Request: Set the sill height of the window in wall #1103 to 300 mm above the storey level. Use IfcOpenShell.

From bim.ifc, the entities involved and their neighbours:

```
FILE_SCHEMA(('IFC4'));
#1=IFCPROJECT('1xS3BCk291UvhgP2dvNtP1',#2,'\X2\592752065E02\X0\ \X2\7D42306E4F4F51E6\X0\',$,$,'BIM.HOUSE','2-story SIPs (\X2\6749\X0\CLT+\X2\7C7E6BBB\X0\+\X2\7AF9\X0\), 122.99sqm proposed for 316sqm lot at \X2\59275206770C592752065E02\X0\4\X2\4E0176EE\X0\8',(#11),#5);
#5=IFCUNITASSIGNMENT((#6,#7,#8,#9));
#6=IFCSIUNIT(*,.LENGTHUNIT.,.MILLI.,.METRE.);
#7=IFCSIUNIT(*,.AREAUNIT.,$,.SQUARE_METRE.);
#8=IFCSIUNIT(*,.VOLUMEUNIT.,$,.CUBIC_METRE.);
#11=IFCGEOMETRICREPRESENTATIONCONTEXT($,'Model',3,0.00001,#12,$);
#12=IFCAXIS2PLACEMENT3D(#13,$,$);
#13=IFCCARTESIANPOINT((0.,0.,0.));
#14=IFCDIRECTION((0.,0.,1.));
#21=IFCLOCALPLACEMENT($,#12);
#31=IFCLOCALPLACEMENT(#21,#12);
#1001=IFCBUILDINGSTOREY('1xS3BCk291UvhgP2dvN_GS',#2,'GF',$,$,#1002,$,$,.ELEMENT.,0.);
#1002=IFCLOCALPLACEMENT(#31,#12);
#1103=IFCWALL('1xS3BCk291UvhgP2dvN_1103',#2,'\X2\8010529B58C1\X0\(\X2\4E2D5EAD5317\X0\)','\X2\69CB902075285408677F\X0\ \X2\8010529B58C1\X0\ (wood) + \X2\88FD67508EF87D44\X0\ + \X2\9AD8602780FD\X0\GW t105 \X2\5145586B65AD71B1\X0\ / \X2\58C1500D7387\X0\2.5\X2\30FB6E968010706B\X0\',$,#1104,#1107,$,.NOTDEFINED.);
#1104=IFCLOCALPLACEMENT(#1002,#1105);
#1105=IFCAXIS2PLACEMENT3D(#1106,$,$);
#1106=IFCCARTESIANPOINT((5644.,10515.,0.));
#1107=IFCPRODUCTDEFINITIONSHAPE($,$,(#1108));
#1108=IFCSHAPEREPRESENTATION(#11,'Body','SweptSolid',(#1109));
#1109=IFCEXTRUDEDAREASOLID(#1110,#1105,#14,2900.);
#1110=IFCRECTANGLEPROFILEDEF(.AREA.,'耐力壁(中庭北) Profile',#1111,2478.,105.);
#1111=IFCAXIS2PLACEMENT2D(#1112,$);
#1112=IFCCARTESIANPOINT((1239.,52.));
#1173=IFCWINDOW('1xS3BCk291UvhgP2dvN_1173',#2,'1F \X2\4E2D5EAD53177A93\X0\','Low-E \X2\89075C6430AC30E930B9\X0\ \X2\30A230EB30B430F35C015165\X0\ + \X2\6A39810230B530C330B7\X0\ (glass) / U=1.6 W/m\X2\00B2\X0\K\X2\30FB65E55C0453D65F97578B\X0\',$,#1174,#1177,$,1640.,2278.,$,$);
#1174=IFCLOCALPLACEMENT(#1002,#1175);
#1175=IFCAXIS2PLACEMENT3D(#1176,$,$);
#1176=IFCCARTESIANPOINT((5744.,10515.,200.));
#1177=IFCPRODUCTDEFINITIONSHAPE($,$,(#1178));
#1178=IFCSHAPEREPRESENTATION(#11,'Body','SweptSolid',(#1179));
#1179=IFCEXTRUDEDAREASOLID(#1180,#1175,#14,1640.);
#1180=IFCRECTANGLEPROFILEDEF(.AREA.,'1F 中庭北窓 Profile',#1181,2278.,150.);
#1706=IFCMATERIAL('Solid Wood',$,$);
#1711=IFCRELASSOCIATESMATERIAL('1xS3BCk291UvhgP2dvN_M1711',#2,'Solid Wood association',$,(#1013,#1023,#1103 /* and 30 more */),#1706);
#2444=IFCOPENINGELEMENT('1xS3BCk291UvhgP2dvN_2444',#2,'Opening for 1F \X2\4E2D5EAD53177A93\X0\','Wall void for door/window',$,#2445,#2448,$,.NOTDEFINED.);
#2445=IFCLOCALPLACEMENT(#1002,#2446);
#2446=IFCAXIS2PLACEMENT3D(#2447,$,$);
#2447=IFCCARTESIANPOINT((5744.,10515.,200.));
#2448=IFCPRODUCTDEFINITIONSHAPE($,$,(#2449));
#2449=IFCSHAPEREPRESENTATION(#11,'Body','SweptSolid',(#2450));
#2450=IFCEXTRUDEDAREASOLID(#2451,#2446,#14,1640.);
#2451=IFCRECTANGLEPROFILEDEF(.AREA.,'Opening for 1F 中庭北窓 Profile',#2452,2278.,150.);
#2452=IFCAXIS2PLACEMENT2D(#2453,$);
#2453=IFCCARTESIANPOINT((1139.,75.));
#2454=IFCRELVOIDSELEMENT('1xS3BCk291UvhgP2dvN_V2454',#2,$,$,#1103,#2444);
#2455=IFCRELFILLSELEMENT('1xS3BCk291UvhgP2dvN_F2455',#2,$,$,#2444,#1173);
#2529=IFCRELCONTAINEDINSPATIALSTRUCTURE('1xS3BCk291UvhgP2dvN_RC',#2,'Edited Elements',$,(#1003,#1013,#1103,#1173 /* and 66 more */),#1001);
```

```python
import numpy as np
import ifcopenshell
import ifcopenshell.api.geometry
import ifcopenshell.geom
import ifcopenshell.util.element
import ifcopenshell.util.placement
import ifcopenshell.util.shape
import ifcopenshell.util.unit

model = ifcopenshell.open("bim.ifc")
unit_scale = ifcopenshell.util.unit.calculate_unit_scale(model)

window = model.by_guid("1xS3BCk291UvhgP2dvN_1173")
opening = window.FillsVoids[0].RelatingOpeningElement
storey = ifcopenshell.util.element.get_container(window, ifc_class="IfcBuildingStorey")
level = ifcopenshell.util.placement.get_local_placement(storey.ObjectPlacement)[2, 3]

# The opening's origin need not be at the sill, so measure its lowest point.
shape = ifcopenshell.geom.create_shape(ifcopenshell.geom.settings(), opening)
bottom = ifcopenshell.util.shape.get_shape_bottom_elevation(shape, shape.geometry) / unit_scale
dz = level + 0.3 / unit_scale - bottom

shift = np.array([0.0, 0.0, dz])
# The window is not placed relative to its opening, so move both.
for product in (opening, window):
    matrix = ifcopenshell.util.placement.get_local_placement(product.ObjectPlacement)
    matrix[:3, 3] += shift
    ifcopenshell.api.geometry.edit_object_placement(model, product=product, matrix=matrix, is_si=False)

print(f"moved by {dz * unit_scale:+.3f} m")

model.write("bim-out.ifc")
```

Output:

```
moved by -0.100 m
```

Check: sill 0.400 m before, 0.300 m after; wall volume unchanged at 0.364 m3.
